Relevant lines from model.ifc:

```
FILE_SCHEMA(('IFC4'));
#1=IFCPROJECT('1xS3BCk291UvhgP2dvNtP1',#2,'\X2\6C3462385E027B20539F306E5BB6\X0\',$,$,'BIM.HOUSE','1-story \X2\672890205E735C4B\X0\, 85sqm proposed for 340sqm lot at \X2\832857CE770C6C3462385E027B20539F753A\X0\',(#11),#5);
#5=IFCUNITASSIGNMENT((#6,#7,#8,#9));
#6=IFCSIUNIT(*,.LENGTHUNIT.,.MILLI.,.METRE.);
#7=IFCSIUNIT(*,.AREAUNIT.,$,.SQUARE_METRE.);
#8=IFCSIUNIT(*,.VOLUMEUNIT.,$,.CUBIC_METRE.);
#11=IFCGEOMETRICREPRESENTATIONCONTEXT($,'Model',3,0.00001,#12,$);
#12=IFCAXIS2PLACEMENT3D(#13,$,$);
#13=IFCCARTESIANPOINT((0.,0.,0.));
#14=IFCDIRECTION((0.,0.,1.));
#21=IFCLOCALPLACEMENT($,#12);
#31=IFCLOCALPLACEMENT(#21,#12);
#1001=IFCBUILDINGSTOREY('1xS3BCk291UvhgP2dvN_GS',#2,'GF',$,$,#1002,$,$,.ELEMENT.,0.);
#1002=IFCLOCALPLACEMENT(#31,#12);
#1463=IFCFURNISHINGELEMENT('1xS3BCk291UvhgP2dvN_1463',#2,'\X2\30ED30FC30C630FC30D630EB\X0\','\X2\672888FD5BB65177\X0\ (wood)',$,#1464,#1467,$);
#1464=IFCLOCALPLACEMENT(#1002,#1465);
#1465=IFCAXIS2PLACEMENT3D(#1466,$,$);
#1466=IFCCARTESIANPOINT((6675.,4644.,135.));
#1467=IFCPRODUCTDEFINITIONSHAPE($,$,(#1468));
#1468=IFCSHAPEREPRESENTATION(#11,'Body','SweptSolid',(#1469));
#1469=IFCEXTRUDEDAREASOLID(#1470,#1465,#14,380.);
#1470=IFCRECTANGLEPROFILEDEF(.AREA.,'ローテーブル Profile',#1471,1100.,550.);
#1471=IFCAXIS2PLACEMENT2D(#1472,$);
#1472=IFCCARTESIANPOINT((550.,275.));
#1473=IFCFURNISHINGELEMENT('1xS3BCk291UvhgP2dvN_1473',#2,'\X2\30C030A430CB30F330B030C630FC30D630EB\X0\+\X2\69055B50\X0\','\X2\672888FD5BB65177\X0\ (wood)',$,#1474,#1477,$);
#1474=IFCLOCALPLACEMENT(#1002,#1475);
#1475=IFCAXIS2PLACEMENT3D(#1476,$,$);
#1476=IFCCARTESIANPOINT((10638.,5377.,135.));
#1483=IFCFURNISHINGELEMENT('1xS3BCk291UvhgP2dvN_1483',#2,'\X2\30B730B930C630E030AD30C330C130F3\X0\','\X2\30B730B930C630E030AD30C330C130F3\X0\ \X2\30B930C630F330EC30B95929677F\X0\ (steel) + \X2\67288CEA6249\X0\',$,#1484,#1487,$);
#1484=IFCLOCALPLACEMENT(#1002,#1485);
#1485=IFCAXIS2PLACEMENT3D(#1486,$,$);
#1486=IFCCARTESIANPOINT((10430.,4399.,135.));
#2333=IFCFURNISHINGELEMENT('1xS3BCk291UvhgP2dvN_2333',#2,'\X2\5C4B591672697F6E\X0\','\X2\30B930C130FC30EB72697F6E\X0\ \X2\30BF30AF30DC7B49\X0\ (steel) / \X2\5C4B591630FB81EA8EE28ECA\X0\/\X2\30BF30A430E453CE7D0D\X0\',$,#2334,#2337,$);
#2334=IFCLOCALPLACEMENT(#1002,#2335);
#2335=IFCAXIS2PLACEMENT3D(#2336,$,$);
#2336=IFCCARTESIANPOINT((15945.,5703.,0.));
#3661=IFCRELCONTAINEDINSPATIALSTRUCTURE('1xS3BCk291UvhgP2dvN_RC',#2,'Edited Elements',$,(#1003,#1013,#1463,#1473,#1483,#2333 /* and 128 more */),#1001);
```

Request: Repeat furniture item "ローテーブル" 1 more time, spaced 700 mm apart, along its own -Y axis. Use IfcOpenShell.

```python
import ifcopenshell
import ifcopenshell.api.geometry
import ifcopenshell.api.root
import ifcopenshell.util.element
import ifcopenshell.util.placement
import ifcopenshell.util.unit

model = ifcopenshell.open("model.ifc")
unit_scale = ifcopenshell.util.unit.calculate_unit_scale(model)


def reuse_history(source, copy):
    """copy_class also copies each property set's owner history, people and application; keep the originals."""
    for rel in copy.IsDefinedBy:
        if rel.is_a("IfcRelDefinesByProperties") and (history := rel.RelatingPropertyDefinition.OwnerHistory):
            rel.RelatingPropertyDefinition.OwnerHistory = source.OwnerHistory
            ifcopenshell.util.element.remove_deep2(model, history)


source = model.by_guid("1xS3BCk291UvhgP2dvN_1463")
base = ifcopenshell.util.placement.get_local_placement(source.ObjectPlacement)
step = -base[:3, 1] * 0.7 / unit_scale

for i in range(1, 2):
    copy = ifcopenshell.api.root.copy_class(model, product=source)
    copy.Representation = ifcopenshell.util.element.copy_deep(
        model, source.Representation, exclude=["IfcGeometricRepresentationContext", "IfcRepresentationMap"]
    )
    reuse_history(source, copy)
    matrix = base.copy()
    matrix[:3, 3] += i * step
    print("added at", matrix[:3, 3].round(3) + 0.0)
    ifcopenshell.api.geometry.edit_object_placement(model, product=copy, matrix=matrix, is_si=False)

model.write("model_edited.ifc")
```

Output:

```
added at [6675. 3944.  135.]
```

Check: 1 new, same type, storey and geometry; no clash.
